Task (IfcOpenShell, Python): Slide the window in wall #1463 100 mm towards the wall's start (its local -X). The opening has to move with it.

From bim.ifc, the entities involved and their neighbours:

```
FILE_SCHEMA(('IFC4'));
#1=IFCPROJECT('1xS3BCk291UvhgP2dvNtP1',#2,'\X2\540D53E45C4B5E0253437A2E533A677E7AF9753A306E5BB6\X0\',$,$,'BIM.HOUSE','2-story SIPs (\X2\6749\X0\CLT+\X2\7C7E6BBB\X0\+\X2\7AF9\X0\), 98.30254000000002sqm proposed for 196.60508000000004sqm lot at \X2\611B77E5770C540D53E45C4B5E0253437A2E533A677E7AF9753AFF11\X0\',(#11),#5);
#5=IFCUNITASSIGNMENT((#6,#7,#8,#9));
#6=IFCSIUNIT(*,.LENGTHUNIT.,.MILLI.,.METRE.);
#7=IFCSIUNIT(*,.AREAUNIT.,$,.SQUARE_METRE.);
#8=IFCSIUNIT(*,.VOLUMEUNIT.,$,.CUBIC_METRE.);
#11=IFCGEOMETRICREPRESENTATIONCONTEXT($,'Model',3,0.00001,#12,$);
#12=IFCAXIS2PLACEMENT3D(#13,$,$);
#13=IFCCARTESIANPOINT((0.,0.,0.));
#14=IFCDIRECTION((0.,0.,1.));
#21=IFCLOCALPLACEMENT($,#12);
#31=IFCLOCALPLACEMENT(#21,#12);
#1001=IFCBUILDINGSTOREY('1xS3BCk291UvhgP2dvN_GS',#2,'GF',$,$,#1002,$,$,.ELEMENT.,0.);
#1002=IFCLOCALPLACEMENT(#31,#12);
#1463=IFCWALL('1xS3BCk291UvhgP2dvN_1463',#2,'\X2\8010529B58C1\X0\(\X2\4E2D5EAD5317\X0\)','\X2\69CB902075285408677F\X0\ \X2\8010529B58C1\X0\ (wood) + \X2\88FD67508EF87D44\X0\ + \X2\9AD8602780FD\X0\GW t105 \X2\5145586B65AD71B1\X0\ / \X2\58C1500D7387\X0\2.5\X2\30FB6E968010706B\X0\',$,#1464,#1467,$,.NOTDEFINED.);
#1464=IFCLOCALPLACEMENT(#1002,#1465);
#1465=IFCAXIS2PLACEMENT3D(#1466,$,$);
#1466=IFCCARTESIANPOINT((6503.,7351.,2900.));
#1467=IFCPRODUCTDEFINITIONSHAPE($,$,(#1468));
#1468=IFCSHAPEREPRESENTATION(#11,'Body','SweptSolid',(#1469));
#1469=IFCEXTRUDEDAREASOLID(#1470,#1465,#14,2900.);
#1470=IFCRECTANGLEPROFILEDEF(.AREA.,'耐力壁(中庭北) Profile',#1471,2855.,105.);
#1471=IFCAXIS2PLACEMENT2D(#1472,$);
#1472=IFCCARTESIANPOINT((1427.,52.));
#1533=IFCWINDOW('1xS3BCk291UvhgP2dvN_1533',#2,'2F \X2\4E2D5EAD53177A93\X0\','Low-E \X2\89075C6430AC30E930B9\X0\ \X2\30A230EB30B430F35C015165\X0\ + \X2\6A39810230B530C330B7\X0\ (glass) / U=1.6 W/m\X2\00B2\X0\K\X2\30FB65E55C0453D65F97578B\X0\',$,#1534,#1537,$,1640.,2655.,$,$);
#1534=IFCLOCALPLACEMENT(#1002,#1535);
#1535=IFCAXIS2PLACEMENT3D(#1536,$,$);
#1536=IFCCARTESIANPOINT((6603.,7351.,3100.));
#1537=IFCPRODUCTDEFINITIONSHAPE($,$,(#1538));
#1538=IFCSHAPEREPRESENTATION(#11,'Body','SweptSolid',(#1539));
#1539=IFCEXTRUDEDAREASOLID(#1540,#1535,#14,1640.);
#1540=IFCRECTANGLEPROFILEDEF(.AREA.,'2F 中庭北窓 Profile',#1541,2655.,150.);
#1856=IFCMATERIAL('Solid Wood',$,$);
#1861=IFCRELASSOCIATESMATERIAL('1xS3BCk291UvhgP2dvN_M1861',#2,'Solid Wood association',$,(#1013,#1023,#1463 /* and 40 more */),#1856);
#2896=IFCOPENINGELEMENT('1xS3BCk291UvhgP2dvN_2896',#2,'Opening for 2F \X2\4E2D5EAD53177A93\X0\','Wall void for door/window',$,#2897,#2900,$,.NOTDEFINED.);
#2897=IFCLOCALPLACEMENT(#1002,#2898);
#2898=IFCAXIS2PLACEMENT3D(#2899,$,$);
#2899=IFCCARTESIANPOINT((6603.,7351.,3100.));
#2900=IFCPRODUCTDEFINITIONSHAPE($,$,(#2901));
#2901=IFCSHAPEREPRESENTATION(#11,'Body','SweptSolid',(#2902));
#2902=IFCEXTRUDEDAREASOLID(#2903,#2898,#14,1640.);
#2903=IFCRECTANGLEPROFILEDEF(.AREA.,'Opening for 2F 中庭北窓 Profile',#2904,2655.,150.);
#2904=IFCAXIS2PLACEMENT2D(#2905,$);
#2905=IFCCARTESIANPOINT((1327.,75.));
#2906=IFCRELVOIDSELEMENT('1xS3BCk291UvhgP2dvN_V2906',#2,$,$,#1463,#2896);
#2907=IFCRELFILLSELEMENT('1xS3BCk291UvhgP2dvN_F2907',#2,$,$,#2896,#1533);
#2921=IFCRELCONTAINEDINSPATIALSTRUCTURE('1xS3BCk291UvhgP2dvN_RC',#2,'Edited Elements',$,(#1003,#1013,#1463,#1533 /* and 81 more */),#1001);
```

```python
import ifcopenshell
import ifcopenshell.api.geometry
import ifcopenshell.util.placement
import ifcopenshell.util.unit

model = ifcopenshell.open("bim.ifc")
unit_scale = ifcopenshell.util.unit.calculate_unit_scale(model)

window = model.by_guid("1xS3BCk291UvhgP2dvN_1533")
opening = window.FillsVoids[0].RelatingOpeningElement
wall = opening.VoidsElements[0].RelatingBuildingElement

wall_matrix = ifcopenshell.util.placement.get_local_placement(wall.ObjectPlacement)
shift = wall_matrix[:3, 0] * -0.1 / unit_scale
before = ifcopenshell.util.placement.get_local_placement(window.ObjectPlacement)[:3, 3].copy()

# The window is not placed relative to its opening, so move both.
for product in (opening, window):
    matrix = ifcopenshell.util.placement.get_local_placement(product.ObjectPlacement)
    matrix[:3, 3] += shift
    ifcopenshell.api.geometry.edit_object_placement(model, product=product, matrix=matrix, is_si=False)

after = ifcopenshell.util.placement.get_local_placement(window.ObjectPlacement)[:3, 3]
print("window moved by", (after - before).round(3) + 0.0)

model.write("bim_rev.ifc")
```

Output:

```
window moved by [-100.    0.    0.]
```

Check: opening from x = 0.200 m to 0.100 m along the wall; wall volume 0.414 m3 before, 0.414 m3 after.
